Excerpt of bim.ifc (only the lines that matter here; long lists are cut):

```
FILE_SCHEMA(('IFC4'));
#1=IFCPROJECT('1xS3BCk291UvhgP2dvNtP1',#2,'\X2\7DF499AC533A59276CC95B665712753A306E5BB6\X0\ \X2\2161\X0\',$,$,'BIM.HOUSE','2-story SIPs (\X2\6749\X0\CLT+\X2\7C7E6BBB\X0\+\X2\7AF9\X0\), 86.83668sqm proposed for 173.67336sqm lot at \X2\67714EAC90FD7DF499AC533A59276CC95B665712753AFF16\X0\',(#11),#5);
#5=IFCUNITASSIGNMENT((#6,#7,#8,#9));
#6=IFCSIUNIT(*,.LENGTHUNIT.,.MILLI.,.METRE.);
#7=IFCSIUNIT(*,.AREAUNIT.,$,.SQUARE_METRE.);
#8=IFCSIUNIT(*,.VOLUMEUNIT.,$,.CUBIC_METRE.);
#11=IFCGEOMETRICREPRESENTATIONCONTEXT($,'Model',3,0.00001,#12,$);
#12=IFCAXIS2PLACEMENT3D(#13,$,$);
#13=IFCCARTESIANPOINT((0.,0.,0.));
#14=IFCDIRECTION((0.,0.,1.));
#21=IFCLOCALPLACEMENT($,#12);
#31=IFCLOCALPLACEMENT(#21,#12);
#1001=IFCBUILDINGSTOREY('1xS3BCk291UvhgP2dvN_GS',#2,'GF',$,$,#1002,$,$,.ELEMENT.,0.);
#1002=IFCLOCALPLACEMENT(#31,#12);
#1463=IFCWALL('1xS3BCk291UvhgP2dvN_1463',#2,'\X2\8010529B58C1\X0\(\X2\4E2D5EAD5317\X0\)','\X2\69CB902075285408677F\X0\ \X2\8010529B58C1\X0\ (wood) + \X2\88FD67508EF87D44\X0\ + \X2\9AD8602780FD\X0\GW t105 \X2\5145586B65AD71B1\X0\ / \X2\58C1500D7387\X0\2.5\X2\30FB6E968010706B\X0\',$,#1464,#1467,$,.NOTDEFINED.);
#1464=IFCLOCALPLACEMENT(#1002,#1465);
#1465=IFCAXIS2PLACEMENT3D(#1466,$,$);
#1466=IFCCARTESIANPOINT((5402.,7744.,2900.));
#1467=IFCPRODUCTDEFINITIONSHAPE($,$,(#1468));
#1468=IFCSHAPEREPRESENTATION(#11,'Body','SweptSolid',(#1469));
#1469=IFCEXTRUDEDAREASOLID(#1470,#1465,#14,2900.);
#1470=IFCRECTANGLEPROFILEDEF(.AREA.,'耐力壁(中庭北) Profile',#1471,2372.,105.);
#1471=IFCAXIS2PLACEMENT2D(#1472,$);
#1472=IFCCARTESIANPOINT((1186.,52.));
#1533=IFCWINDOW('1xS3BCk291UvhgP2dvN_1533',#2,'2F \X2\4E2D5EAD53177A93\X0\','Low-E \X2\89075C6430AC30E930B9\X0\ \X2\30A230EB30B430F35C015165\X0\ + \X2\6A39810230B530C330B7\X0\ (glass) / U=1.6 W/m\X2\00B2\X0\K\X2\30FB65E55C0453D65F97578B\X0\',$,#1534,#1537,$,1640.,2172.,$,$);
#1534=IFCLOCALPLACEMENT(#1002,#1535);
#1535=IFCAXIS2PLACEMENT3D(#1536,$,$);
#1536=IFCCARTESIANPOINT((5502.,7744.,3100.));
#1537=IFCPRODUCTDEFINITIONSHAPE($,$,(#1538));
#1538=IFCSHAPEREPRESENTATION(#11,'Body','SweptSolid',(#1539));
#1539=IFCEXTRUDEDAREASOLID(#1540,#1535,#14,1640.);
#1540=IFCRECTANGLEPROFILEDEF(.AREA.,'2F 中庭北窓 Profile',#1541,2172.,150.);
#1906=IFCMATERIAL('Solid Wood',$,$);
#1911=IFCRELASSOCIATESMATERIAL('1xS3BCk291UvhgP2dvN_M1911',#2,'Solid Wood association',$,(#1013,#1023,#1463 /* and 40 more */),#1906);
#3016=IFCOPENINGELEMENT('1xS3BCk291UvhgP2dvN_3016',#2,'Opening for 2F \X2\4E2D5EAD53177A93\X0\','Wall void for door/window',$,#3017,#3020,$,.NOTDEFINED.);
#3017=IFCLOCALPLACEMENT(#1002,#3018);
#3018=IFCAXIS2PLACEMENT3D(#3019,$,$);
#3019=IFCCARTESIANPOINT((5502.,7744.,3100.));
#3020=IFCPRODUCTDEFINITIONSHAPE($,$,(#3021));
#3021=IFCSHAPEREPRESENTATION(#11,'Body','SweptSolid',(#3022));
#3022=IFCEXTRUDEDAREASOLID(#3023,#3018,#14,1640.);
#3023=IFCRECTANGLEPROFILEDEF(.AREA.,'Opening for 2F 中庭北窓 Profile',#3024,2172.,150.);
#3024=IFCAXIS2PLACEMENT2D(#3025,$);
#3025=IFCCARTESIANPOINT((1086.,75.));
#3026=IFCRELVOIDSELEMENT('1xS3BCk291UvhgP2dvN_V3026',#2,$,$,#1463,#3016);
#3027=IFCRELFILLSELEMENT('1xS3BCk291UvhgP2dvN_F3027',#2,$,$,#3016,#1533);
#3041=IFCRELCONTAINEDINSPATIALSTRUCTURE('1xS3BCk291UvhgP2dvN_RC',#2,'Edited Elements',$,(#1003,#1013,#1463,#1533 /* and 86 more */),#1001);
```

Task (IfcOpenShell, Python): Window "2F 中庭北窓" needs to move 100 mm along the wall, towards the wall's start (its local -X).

```python
import ifcopenshell
import ifcopenshell.api.geometry
import ifcopenshell.util.placement

model = ifcopenshell.open("bim.ifc")

window = model.by_guid("1xS3BCk291UvhgP2dvN_1533")
opening = window.FillsVoids[0].RelatingOpeningElement
wall = opening.VoidsElements[0].RelatingBuildingElement

wall_matrix = ifcopenshell.util.placement.get_local_placement(wall.ObjectPlacement)
shift = wall_matrix[:3, 0] * -100.0
before = ifcopenshell.util.placement.get_local_placement(window.ObjectPlacement)[:3, 3].copy()

# The window is not placed relative to its opening, so move both.
for product in (opening, window):
    matrix = ifcopenshell.util.placement.get_local_placement(product.ObjectPlacement)
    matrix[:3, 3] += shift
    ifcopenshell.api.geometry.edit_object_placement(model, product=product, matrix=matrix, is_si=False)

after = ifcopenshell.util.placement.get_local_placement(window.ObjectPlacement)[:3, 3]
print("window moved by", (after - before).round(3) + 0.0)

model.write("bim_rev.ifc")
```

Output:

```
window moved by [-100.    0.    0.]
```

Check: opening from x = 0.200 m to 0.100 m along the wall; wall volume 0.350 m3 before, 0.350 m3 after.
